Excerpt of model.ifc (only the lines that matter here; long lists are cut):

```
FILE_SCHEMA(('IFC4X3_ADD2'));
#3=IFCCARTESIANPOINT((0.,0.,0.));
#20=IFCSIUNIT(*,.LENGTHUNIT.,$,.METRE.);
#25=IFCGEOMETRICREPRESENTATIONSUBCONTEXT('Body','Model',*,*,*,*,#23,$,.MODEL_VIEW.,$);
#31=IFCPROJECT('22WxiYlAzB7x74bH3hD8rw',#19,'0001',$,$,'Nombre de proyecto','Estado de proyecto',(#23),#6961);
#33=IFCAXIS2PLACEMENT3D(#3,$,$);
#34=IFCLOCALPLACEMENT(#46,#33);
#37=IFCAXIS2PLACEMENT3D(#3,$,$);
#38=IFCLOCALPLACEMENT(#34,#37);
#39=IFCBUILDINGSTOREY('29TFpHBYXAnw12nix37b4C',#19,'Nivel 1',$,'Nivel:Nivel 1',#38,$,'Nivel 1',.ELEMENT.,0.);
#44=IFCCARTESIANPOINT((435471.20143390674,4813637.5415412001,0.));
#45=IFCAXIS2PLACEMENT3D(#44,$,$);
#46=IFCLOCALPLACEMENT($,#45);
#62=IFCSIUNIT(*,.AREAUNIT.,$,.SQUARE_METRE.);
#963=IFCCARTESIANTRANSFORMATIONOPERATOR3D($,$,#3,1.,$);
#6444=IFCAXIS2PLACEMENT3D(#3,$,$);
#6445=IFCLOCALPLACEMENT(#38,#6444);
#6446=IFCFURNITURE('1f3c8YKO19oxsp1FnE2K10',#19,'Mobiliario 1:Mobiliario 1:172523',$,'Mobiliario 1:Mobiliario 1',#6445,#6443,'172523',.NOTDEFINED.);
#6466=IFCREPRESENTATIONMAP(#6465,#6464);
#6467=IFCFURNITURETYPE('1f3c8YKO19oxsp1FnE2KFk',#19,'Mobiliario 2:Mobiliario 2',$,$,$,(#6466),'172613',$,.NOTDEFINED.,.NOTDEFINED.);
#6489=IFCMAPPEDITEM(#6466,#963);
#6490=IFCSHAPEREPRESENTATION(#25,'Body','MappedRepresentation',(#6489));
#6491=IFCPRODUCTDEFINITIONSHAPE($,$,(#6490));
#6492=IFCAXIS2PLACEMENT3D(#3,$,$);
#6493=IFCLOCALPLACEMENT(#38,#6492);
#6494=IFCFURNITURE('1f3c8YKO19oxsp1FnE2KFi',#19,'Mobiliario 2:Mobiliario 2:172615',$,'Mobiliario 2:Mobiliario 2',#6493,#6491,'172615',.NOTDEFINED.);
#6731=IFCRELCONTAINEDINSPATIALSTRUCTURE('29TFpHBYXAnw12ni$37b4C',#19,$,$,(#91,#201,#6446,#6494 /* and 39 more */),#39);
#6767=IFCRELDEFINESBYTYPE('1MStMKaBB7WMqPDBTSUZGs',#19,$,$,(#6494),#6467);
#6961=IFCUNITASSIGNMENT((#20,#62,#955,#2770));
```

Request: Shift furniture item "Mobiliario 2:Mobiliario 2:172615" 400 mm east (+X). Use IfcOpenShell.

```python
import ifcopenshell
import ifcopenshell.api.geometry
import ifcopenshell.util.placement

model = ifcopenshell.open("model.ifc")

item = model.by_guid("1f3c8YKO19oxsp1FnE2KFi")
matrix = ifcopenshell.util.placement.get_local_placement(item.ObjectPlacement)
matrix[0, 3] += 0.4
ifcopenshell.api.geometry.edit_object_placement(model, product=item, matrix=matrix, is_si=False)

print(ifcopenshell.util.placement.get_local_placement(item.ObjectPlacement).round(3) + 0.0)

model.write("model_v2.ifc")
```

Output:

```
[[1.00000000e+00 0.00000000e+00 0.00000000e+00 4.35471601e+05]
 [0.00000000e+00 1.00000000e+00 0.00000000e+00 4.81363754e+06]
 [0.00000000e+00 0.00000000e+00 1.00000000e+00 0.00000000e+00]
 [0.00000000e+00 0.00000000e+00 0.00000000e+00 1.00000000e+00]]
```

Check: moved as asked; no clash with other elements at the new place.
